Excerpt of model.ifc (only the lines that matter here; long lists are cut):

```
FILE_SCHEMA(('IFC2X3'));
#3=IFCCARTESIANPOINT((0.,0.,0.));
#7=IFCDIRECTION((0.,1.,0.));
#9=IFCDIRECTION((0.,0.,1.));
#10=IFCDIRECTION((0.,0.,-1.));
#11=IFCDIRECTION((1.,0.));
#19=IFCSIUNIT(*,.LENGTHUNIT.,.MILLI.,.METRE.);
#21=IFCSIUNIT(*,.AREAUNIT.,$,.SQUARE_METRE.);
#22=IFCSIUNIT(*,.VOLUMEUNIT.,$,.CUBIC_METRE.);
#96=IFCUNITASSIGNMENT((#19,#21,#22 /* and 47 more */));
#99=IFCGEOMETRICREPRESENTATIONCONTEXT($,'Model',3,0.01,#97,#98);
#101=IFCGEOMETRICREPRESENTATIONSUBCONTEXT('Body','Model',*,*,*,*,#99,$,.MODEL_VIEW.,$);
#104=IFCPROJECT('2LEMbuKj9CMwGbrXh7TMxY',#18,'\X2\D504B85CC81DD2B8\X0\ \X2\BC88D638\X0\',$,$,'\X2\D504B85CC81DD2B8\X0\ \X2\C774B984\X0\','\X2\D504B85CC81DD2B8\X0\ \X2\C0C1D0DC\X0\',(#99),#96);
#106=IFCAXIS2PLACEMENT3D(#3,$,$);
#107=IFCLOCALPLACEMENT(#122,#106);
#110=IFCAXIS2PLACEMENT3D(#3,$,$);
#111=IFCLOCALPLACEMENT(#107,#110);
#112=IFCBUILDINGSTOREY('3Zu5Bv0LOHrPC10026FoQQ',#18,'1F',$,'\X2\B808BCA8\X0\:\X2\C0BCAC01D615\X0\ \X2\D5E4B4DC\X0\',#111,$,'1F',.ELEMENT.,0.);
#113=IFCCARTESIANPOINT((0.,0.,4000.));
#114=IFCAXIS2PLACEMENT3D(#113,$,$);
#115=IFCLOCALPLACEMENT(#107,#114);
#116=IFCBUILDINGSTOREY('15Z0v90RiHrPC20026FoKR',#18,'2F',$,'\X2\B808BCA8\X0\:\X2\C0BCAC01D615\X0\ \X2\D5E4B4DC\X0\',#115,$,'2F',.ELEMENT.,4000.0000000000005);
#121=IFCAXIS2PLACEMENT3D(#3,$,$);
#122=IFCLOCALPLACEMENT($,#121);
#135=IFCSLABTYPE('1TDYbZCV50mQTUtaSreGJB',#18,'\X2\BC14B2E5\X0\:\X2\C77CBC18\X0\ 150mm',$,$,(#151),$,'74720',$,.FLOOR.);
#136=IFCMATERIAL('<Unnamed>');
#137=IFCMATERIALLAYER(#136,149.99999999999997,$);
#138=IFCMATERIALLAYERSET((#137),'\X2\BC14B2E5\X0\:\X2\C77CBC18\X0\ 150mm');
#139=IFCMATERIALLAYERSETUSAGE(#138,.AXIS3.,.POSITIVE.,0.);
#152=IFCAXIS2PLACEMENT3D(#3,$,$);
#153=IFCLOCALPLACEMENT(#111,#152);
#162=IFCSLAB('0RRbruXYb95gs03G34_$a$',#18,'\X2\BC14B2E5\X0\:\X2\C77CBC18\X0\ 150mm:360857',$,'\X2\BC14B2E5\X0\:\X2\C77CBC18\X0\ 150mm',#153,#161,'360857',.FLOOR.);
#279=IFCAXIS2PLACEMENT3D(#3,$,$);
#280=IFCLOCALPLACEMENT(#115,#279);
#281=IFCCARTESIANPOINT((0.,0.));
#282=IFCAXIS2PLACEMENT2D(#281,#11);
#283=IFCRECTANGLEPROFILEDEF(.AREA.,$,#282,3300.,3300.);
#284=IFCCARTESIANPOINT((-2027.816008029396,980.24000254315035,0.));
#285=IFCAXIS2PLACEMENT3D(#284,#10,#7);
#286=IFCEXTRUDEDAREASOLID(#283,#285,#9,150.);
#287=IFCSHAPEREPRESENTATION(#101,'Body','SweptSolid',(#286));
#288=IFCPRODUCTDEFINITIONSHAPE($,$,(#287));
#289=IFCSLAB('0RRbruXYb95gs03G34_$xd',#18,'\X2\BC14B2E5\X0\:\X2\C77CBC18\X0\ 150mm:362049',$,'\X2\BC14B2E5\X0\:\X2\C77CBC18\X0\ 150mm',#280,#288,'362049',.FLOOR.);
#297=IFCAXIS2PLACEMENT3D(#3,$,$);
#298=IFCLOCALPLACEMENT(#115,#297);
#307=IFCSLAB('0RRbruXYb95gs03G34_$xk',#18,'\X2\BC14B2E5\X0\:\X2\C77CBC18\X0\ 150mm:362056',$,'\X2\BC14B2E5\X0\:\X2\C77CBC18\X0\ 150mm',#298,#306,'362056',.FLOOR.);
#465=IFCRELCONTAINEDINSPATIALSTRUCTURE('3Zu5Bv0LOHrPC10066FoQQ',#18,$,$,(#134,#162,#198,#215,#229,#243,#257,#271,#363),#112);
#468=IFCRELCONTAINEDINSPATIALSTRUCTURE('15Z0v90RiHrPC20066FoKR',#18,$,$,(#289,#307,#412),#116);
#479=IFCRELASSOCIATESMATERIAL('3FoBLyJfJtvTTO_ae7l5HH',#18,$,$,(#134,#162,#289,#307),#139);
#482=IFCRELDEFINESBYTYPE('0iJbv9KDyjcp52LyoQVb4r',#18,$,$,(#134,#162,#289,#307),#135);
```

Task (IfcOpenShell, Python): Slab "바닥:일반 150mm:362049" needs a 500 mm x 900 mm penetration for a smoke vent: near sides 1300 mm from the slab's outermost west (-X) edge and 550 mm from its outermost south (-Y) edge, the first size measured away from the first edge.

```python
import numpy as np
import ifcopenshell
import ifcopenshell.api.feature
import ifcopenshell.api.geometry
import ifcopenshell.api.root
import ifcopenshell.geom
import ifcopenshell.util.placement
import ifcopenshell.util.representation
import ifcopenshell.util.shape
import ifcopenshell.util.unit

model = ifcopenshell.open("model.ifc")
unit_scale = ifcopenshell.util.unit.calculate_unit_scale(model)
settings = ifcopenshell.geom.settings()


def volume(element):
    """Net volume in cubic metres, openings subtracted."""
    shape = ifcopenshell.geom.create_shape(settings, element)
    return ifcopenshell.util.shape.get_volume(shape.geometry)


slab = model.by_id(289)
before = volume(slab)

# Extent in the slab's own axes, in metres. The edges named are its -X and -Y sides.
slab_shape = ifcopenshell.geom.create_shape(settings, slab)
vertices = ifcopenshell.util.shape.get_vertices(slab_shape.geometry)
x_min, y_min, bottom = vertices.min(axis=0)
top = vertices[:, 2].max()

opening = ifcopenshell.api.root.create_entity(model, ifc_class="IfcOpeningElement", name="Smoke vent opening")
context = ifcopenshell.util.representation.get_context(model, "Model", "Body", "MODEL_VIEW")
width, depth = 0.5, 0.9
outline = [(0.0, 0.0), (width, 0.0), (width, depth), (0.0, depth), (0.0, 0.0)]
# Overshoot both faces by 50 mm so the cut is clean.
shape = ifcopenshell.api.geometry.add_slab_representation(
    model, context=context, depth=top - bottom + 0.1, polyline=outline
)
ifcopenshell.api.geometry.assign_representation(model, product=opening, representation=shape)

matrix = ifcopenshell.util.placement.get_local_placement(slab.ObjectPlacement)
matrix[:, 3] = matrix @ np.append(np.array([x_min + 1.3, y_min + 0.55, bottom - 0.05]) / unit_scale, 1.0)
ifcopenshell.api.geometry.edit_object_placement(model, product=opening, matrix=matrix, is_si=False)
ifcopenshell.api.feature.add_feature(model, feature=opening, element=slab)

after = volume(slab)

print(f"slab volume {before:.3f} -> {after:.3f} m3")

model.write("model-out.ifc")
```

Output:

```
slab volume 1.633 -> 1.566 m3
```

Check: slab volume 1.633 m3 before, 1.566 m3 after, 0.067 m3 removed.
